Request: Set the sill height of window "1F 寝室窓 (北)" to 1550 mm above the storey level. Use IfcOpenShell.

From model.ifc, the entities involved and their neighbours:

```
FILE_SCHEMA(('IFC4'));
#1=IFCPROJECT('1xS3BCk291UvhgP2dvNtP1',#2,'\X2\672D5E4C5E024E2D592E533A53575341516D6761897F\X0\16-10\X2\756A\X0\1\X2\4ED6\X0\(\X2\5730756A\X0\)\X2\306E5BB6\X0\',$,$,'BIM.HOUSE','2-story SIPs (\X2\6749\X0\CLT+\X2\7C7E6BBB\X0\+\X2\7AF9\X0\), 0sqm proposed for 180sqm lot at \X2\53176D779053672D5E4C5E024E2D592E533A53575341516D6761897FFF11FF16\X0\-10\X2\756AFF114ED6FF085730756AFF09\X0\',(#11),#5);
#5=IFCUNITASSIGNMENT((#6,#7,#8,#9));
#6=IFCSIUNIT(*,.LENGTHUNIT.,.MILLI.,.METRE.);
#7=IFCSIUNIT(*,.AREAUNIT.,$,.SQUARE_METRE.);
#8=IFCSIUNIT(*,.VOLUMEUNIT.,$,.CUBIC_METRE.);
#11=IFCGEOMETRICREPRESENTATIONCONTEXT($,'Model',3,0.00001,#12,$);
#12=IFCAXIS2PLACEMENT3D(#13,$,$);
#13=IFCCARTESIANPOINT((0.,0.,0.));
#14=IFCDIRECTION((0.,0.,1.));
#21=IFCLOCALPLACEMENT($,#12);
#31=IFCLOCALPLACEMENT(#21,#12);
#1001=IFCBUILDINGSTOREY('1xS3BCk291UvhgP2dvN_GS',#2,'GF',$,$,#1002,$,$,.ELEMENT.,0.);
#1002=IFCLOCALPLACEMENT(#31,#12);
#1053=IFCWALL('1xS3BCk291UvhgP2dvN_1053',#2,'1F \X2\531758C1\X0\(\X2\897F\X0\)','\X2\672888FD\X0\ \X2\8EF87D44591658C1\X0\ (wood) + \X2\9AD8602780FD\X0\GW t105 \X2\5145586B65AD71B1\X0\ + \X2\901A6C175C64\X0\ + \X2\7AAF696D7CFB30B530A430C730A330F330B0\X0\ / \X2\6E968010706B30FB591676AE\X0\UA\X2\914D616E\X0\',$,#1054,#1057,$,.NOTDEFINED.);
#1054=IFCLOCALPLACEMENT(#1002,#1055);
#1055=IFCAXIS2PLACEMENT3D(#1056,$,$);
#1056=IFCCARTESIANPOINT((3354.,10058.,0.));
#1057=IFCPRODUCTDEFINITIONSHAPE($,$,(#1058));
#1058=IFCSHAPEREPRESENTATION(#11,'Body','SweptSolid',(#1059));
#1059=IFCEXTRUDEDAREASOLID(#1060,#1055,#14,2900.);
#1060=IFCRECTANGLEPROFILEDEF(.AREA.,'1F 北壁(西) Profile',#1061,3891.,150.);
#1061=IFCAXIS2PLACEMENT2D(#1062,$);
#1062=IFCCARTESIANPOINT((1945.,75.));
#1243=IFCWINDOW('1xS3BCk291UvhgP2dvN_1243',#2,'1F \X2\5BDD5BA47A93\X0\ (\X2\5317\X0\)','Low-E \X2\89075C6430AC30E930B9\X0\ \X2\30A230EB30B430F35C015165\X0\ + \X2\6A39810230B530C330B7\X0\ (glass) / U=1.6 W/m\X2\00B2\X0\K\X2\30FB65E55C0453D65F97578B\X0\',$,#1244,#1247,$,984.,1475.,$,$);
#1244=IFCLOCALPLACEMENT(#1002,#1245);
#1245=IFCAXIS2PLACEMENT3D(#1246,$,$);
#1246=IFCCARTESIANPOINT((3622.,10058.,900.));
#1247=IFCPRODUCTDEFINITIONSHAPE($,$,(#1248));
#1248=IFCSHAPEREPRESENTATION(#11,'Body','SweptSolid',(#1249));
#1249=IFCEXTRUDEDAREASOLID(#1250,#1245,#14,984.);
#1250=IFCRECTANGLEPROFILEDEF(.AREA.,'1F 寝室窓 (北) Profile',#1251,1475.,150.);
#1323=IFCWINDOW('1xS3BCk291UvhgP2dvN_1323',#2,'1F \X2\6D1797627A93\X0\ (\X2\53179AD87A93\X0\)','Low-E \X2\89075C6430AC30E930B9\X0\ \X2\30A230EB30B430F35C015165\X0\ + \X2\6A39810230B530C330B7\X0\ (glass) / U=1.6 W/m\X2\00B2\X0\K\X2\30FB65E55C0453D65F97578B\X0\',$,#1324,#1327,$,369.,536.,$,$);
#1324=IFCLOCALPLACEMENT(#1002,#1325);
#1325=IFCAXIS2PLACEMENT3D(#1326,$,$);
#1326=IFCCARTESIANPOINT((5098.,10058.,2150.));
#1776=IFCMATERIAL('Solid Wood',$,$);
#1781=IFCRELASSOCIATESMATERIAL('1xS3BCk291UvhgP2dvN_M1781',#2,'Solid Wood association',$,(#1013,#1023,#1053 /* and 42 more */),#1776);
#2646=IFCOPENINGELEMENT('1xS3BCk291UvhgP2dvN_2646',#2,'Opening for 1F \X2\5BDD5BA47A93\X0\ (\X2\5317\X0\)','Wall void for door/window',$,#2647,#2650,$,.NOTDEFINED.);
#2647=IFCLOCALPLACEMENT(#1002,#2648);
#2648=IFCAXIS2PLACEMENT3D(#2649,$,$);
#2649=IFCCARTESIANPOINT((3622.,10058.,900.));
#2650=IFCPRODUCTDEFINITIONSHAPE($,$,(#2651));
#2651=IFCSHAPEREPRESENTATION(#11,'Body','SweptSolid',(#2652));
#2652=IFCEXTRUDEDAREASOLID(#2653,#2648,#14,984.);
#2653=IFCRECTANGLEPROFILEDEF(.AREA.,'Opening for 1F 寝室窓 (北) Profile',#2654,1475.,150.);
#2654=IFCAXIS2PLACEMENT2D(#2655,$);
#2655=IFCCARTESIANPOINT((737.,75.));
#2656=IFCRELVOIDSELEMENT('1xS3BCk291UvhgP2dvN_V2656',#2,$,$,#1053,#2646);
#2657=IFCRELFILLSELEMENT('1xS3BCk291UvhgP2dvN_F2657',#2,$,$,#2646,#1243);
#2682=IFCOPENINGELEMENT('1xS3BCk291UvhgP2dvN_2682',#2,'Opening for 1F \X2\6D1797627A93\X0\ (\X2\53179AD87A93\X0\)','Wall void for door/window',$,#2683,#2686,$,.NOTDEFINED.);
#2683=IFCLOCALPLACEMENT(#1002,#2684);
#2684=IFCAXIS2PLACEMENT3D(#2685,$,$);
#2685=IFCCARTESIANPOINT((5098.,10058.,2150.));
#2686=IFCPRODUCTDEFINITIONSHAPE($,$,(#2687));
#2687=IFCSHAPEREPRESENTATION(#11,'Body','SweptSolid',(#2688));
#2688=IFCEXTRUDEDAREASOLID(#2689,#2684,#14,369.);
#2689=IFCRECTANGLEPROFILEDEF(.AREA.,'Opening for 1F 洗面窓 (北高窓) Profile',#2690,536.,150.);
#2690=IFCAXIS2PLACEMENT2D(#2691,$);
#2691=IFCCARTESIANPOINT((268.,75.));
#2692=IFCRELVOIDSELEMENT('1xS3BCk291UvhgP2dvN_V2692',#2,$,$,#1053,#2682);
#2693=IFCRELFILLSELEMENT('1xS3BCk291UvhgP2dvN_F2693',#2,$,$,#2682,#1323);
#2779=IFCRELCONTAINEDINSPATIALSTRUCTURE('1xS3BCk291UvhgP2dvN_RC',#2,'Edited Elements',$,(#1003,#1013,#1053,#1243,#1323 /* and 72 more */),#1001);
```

```python
import numpy as np
import ifcopenshell
import ifcopenshell.api.geometry
import ifcopenshell.geom
import ifcopenshell.util.element
import ifcopenshell.util.placement
import ifcopenshell.util.shape
import ifcopenshell.util.unit

model = ifcopenshell.open("model.ifc")
unit_scale = ifcopenshell.util.unit.calculate_unit_scale(model)

window = model.by_id(1243)
opening = window.FillsVoids[0].RelatingOpeningElement
storey = ifcopenshell.util.element.get_container(window, ifc_class="IfcBuildingStorey")
level = ifcopenshell.util.placement.get_local_placement(storey.ObjectPlacement)[2, 3]

# The opening's origin need not be at the sill, so measure its lowest point.
shape = ifcopenshell.geom.create_shape(ifcopenshell.geom.settings(), opening)
bottom = ifcopenshell.util.shape.get_shape_bottom_elevation(shape, shape.geometry) / unit_scale
dz = level + 1550.0 - bottom

shift = np.array([0.0, 0.0, dz])
# The window is not placed relative to its opening, so move both.
for product in (opening, window):
    matrix = ifcopenshell.util.placement.get_local_placement(product.ObjectPlacement)
    matrix[:3, 3] += shift
    ifcopenshell.api.geometry.edit_object_placement(model, product=product, matrix=matrix, is_si=False)

print(f"moved by {dz * unit_scale:+.3f} m")

model.write("model_rev.ifc")
```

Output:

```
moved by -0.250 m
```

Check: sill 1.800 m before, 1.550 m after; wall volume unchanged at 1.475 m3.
